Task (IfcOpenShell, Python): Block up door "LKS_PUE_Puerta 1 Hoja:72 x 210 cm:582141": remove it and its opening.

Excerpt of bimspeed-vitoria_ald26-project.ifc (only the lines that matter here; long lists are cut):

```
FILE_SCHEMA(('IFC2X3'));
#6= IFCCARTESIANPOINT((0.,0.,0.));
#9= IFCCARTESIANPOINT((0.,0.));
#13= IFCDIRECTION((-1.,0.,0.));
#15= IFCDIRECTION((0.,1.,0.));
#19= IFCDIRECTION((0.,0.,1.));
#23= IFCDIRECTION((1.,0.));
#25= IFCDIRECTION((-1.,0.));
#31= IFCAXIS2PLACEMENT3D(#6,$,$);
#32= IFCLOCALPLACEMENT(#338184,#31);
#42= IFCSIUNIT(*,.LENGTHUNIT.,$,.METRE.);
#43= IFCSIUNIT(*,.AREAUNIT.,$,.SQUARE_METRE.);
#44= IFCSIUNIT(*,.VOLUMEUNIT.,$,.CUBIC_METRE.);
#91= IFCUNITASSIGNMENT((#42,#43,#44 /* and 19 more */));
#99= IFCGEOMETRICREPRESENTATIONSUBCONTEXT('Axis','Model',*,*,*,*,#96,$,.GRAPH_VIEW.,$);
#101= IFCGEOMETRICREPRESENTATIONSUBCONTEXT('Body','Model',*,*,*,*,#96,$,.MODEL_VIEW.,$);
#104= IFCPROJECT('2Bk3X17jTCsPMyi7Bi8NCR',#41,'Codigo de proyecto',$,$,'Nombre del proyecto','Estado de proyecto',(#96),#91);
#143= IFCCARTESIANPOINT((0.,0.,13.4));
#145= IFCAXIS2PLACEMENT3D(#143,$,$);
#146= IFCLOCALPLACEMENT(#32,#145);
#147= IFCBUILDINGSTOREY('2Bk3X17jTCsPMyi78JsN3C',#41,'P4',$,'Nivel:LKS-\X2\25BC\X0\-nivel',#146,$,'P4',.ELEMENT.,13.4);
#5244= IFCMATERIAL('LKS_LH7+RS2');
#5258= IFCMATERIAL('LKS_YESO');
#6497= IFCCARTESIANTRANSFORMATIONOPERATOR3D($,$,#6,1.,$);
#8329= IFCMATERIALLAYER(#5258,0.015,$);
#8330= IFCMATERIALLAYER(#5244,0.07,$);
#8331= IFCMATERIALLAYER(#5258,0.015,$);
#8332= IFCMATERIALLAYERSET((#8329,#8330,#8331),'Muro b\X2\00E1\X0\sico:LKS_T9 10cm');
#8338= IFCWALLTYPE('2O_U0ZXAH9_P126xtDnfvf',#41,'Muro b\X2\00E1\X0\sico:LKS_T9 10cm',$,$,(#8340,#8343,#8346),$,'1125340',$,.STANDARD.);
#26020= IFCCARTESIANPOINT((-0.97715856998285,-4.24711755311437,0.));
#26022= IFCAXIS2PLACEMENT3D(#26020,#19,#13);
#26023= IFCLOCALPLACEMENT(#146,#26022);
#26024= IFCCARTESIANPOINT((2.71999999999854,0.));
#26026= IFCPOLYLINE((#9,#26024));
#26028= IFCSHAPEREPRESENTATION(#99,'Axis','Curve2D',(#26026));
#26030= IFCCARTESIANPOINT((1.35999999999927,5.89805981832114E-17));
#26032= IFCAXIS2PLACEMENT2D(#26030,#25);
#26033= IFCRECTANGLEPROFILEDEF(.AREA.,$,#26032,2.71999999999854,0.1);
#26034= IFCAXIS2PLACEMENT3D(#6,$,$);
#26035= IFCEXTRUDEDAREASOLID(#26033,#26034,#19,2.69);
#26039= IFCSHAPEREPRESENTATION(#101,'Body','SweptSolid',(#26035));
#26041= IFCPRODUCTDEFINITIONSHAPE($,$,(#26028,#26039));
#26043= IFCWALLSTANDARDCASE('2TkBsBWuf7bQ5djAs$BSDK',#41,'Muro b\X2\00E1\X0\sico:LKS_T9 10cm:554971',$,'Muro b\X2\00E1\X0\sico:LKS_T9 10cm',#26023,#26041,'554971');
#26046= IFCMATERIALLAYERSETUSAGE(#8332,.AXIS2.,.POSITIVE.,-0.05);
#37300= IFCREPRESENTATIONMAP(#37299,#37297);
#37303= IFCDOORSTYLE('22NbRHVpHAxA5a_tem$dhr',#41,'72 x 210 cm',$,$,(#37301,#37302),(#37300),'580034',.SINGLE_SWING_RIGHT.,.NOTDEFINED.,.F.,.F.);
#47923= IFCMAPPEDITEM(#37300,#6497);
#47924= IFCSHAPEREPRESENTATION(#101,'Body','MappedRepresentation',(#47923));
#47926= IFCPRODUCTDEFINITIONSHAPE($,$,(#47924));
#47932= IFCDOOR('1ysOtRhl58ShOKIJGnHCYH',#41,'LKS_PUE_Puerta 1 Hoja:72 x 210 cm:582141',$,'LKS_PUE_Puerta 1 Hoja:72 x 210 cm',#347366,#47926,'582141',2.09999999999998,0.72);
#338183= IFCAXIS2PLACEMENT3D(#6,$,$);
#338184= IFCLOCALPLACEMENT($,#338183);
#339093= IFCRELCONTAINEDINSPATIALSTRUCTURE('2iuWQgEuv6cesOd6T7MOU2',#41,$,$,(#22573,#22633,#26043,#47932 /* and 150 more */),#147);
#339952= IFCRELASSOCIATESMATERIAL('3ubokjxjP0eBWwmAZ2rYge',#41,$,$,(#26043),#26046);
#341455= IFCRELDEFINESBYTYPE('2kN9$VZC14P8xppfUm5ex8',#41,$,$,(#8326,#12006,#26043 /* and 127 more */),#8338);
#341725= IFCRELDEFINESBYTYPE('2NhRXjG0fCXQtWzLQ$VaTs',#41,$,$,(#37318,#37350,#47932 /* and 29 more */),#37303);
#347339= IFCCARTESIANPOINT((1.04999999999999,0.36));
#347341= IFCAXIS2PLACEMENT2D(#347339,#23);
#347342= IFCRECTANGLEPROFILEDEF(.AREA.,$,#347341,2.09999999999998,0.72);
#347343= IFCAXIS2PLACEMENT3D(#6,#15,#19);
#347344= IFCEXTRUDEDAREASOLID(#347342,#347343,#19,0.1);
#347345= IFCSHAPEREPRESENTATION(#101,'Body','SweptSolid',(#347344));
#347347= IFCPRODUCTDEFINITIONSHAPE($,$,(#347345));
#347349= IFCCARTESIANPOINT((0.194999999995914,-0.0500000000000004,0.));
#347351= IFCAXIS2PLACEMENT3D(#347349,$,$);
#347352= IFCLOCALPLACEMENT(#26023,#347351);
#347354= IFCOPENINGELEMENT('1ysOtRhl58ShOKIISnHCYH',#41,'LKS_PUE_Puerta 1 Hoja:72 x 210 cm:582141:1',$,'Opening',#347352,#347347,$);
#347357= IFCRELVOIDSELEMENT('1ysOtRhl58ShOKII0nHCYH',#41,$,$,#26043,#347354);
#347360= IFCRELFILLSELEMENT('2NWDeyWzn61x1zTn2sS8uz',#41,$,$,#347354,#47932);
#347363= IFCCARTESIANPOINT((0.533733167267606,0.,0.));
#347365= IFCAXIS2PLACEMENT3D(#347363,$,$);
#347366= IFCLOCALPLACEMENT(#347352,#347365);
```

```python
import ifcopenshell
import ifcopenshell.api.feature
import ifcopenshell.api.root
import ifcopenshell.geom
import ifcopenshell.util.shape

model = ifcopenshell.open("bimspeed-vitoria_ald26-project.ifc")
settings = ifcopenshell.geom.settings()


def volume(element):
    """Net volume in cubic metres, openings subtracted."""
    shape = ifcopenshell.geom.create_shape(settings, element)
    return ifcopenshell.util.shape.get_volume(shape.geometry)


door = model.by_id(47932)
opening = door.FillsVoids[0].RelatingOpeningElement
wall = opening.VoidsElements[0].RelatingBuildingElement
before = volume(wall)

ifcopenshell.api.root.remove_product(model, product=door)
ifcopenshell.api.feature.remove_feature(model, feature=opening)

after = volume(wall)

print(f"wall volume {before:.3f} -> {after:.3f} m3")

model.write("bimspeed-vitoria_ald26-project_updated.ifc")
```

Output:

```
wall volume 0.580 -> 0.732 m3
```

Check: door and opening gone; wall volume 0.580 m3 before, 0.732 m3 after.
